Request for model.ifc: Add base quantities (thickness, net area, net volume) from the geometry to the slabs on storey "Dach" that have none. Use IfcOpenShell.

First a look at what the model holds.

```python
import ifcopenshell
import ifcopenshell.util.element
import ifcopenshell.util.unit

model = ifcopenshell.open("model.ifc")
print(model.schema)
for unit_type in ("LENGTHUNIT", "AREAUNIT", "VOLUMEUNIT"):
    print(unit_type, ifcopenshell.util.unit.calculate_unit_scale(model, unit_type))
storey = next(s for s in model.by_type("IfcBuildingStorey") if s.Name == "Dach")
slabs = [e for e in ifcopenshell.util.element.get_decomposition(storey) if e.is_a("IfcSlab")]
for e in sorted(slabs, key=lambda e: e.id()):
    print(e.id(), e.is_a(), e.Name, list(ifcopenshell.util.element.get_psets(e, qtos_only=True)), sep=" | ")
```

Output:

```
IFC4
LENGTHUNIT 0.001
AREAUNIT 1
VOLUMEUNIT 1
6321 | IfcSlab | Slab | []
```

```python
import ifcopenshell
import ifcopenshell.api.pset
import ifcopenshell.geom
import ifcopenshell.util.element
import ifcopenshell.util.shape
import ifcopenshell.util.unit

model = ifcopenshell.open("model.ifc")
unit_scale = ifcopenshell.util.unit.calculate_unit_scale(model)
area_scale = ifcopenshell.util.unit.calculate_unit_scale(model, "AREAUNIT")
volume_scale = ifcopenshell.util.unit.calculate_unit_scale(model, "VOLUMEUNIT")
settings = ifcopenshell.geom.settings()

storey = next(s for s in model.by_type("IfcBuildingStorey") if s.Name == "Dach")
slabs = [e for e in ifcopenshell.util.element.get_decomposition(storey) if e.is_a("IfcSlab")]

for e in sorted(slabs, key=lambda e: e.id()):
    if ifcopenshell.util.element.get_psets(e, qtos_only=True, should_inherit=False):
        continue
    # Geometry comes back in metres, in the element's own axes.
    shape = ifcopenshell.geom.create_shape(settings, e)
    values = {
        "Width": ifcopenshell.util.shape.get_z(shape.geometry) / unit_scale,
        "NetArea": ifcopenshell.util.shape.get_footprint_area(shape.geometry) / area_scale,
        "NetVolume": ifcopenshell.util.shape.get_volume(shape.geometry) / volume_scale,
    }
    qto = ifcopenshell.api.pset.add_qto(model, product=e, name="Qto_SlabBaseQuantities")
    ifcopenshell.api.pset.edit_qto(model, qto=qto, properties=values)
    print(e.id(), {k: round(v, 3) for k, v in values.items()})

model.write("model-out.ifc")
```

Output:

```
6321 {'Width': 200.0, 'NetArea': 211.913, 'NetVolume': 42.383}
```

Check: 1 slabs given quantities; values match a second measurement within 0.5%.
